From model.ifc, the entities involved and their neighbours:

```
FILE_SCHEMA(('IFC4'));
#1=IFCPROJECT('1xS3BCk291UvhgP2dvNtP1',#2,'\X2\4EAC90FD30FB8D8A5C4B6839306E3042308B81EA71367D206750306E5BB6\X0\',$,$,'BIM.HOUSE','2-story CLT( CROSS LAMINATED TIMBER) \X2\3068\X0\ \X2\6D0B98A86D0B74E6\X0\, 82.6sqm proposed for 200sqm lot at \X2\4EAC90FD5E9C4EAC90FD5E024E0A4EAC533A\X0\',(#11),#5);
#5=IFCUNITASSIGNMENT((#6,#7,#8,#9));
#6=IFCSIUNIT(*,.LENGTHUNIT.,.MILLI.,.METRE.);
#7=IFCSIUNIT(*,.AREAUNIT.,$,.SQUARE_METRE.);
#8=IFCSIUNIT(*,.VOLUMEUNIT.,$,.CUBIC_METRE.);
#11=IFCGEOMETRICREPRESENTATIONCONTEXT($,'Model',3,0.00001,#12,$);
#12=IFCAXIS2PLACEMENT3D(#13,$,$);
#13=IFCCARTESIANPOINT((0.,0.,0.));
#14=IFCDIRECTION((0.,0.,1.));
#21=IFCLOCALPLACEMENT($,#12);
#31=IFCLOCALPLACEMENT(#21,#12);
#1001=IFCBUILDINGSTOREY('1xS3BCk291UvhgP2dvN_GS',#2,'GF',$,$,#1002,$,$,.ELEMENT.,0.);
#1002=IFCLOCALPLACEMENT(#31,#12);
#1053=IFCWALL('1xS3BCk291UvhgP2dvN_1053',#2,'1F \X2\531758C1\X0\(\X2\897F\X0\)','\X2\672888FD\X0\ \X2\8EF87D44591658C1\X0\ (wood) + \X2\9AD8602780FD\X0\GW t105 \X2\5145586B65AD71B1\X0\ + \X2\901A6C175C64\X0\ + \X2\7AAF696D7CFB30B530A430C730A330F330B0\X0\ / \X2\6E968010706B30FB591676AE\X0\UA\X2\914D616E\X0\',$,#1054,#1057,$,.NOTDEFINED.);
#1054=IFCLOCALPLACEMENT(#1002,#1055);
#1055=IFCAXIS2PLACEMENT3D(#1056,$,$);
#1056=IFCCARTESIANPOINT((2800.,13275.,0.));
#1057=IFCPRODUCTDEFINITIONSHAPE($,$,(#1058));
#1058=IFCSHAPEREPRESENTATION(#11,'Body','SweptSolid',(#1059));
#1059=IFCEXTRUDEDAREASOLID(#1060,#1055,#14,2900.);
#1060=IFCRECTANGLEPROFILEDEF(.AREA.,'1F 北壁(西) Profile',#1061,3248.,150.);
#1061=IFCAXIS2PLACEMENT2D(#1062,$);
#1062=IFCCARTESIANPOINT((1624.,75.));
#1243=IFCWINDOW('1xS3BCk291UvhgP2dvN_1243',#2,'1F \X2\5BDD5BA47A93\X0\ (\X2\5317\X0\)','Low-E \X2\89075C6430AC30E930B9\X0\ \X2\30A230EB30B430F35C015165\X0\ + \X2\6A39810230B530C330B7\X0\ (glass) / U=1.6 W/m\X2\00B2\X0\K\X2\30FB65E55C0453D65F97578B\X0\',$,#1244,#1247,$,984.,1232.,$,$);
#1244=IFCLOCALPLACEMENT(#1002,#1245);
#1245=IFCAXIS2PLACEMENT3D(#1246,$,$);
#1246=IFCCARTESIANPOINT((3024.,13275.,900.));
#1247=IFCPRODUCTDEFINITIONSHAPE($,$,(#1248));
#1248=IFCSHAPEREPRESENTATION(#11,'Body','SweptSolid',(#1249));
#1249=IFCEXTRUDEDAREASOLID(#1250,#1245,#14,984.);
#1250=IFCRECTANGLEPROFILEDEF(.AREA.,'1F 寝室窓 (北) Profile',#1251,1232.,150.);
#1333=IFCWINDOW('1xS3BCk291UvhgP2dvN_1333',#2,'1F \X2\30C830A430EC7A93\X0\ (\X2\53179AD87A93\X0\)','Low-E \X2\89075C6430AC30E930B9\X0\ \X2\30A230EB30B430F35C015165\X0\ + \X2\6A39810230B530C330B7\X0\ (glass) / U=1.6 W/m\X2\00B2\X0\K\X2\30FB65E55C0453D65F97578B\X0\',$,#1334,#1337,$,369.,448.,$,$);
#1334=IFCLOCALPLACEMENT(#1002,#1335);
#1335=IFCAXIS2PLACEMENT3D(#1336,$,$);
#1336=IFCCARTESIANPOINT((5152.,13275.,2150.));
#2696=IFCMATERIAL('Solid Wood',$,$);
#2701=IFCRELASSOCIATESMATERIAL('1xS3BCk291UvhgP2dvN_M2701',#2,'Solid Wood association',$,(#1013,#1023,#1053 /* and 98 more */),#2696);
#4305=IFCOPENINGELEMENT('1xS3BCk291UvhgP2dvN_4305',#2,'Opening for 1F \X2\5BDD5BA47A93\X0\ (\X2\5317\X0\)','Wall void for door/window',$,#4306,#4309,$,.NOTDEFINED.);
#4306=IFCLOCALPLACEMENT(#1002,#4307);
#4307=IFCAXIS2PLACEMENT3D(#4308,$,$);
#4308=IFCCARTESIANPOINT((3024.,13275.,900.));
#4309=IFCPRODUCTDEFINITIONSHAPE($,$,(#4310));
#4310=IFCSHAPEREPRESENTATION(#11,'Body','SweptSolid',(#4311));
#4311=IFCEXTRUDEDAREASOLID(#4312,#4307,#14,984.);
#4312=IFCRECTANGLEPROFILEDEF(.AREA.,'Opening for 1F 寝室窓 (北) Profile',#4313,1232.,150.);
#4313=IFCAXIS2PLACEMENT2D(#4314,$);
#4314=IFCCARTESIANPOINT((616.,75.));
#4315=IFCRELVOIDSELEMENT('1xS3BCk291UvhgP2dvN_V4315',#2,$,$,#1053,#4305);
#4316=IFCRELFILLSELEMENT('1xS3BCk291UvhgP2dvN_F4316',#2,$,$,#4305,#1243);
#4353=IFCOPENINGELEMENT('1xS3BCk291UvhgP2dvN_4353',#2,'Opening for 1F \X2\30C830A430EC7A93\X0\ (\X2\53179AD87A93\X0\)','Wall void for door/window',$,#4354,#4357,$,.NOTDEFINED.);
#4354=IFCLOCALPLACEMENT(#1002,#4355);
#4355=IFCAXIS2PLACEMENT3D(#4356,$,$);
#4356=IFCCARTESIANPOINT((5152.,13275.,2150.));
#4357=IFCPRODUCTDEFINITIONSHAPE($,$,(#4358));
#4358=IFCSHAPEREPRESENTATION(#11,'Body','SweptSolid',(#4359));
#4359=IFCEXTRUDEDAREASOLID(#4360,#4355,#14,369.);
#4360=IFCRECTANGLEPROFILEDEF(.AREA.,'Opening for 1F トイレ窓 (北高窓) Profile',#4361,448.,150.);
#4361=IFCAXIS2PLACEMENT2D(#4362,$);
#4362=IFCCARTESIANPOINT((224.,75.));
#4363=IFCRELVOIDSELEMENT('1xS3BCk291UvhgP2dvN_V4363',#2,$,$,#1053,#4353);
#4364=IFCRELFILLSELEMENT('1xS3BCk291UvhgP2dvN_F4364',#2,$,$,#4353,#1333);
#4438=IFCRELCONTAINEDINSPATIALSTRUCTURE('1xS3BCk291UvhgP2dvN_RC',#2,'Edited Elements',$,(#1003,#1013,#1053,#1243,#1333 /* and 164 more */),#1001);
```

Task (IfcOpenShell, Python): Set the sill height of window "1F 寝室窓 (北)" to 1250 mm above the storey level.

```python
import numpy as np
import ifcopenshell
import ifcopenshell.api.geometry
import ifcopenshell.geom
import ifcopenshell.util.element
import ifcopenshell.util.placement
import ifcopenshell.util.shape
import ifcopenshell.util.unit

model = ifcopenshell.open("model.ifc")
unit_scale = ifcopenshell.util.unit.calculate_unit_scale(model)

window = model.by_guid("1xS3BCk291UvhgP2dvN_1243")
opening = window.FillsVoids[0].RelatingOpeningElement
storey = ifcopenshell.util.element.get_container(window, ifc_class="IfcBuildingStorey")
level = ifcopenshell.util.placement.get_local_placement(storey.ObjectPlacement)[2, 3]

# The opening's origin need not be at the sill, so measure its lowest point.
shape = ifcopenshell.geom.create_shape(ifcopenshell.geom.settings(), opening)
bottom = ifcopenshell.util.shape.get_shape_bottom_elevation(shape, shape.geometry) / unit_scale
dz = level + 1.25 / unit_scale - bottom

shift = np.array([0.0, 0.0, dz])
# The window is not placed relative to its opening, so move both.
for product in (opening, window):
    matrix = ifcopenshell.util.placement.get_local_placement(product.ObjectPlacement)
    matrix[:3, 3] += shift
    ifcopenshell.api.geometry.edit_object_placement(model, product=product, matrix=matrix, is_si=False)

print(f"moved by {dz * unit_scale:+.3f} m")

model.write("model_edited.ifc")
```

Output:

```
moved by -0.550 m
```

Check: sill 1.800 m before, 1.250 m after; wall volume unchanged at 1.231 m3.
